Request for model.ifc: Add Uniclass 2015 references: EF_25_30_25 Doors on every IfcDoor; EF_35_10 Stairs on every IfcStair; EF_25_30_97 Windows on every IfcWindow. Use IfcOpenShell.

First a look at what the model holds.

```python
import ifcopenshell

model = ifcopenshell.open("model.ifc")
print(model.schema)
print("classifications:", [c.Name for c in model.by_type("IfcClassification")])
for ifc_class in ("IfcDoor", "IfcRoof", "IfcStair", "IfcWall", "IfcWindow"):
    print(ifc_class, len(model.by_type(ifc_class)))
```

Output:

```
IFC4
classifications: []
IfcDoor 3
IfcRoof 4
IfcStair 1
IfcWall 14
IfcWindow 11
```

```python
import ifcopenshell
import ifcopenshell.api.classification

model = ifcopenshell.open("model.ifc")

system = ifcopenshell.api.classification.add_classification(model, classification="Uniclass 2015")

codes = {
    "IfcDoor": ("EF_25_30_25", "Doors"),
    "IfcStair": ("EF_35_10", "Stairs"),
    "IfcWindow": ("EF_25_30_97", "Windows"),
}
for ifc_class, (code, name) in codes.items():
    products = model.by_type(ifc_class)
    ifcopenshell.api.classification.add_reference(
        model, products=products, classification=system, identification=code, name=name
    )
    print(code, len(products))

model.write("model_updated.ifc")
```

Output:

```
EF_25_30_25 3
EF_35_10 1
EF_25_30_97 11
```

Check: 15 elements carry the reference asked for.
